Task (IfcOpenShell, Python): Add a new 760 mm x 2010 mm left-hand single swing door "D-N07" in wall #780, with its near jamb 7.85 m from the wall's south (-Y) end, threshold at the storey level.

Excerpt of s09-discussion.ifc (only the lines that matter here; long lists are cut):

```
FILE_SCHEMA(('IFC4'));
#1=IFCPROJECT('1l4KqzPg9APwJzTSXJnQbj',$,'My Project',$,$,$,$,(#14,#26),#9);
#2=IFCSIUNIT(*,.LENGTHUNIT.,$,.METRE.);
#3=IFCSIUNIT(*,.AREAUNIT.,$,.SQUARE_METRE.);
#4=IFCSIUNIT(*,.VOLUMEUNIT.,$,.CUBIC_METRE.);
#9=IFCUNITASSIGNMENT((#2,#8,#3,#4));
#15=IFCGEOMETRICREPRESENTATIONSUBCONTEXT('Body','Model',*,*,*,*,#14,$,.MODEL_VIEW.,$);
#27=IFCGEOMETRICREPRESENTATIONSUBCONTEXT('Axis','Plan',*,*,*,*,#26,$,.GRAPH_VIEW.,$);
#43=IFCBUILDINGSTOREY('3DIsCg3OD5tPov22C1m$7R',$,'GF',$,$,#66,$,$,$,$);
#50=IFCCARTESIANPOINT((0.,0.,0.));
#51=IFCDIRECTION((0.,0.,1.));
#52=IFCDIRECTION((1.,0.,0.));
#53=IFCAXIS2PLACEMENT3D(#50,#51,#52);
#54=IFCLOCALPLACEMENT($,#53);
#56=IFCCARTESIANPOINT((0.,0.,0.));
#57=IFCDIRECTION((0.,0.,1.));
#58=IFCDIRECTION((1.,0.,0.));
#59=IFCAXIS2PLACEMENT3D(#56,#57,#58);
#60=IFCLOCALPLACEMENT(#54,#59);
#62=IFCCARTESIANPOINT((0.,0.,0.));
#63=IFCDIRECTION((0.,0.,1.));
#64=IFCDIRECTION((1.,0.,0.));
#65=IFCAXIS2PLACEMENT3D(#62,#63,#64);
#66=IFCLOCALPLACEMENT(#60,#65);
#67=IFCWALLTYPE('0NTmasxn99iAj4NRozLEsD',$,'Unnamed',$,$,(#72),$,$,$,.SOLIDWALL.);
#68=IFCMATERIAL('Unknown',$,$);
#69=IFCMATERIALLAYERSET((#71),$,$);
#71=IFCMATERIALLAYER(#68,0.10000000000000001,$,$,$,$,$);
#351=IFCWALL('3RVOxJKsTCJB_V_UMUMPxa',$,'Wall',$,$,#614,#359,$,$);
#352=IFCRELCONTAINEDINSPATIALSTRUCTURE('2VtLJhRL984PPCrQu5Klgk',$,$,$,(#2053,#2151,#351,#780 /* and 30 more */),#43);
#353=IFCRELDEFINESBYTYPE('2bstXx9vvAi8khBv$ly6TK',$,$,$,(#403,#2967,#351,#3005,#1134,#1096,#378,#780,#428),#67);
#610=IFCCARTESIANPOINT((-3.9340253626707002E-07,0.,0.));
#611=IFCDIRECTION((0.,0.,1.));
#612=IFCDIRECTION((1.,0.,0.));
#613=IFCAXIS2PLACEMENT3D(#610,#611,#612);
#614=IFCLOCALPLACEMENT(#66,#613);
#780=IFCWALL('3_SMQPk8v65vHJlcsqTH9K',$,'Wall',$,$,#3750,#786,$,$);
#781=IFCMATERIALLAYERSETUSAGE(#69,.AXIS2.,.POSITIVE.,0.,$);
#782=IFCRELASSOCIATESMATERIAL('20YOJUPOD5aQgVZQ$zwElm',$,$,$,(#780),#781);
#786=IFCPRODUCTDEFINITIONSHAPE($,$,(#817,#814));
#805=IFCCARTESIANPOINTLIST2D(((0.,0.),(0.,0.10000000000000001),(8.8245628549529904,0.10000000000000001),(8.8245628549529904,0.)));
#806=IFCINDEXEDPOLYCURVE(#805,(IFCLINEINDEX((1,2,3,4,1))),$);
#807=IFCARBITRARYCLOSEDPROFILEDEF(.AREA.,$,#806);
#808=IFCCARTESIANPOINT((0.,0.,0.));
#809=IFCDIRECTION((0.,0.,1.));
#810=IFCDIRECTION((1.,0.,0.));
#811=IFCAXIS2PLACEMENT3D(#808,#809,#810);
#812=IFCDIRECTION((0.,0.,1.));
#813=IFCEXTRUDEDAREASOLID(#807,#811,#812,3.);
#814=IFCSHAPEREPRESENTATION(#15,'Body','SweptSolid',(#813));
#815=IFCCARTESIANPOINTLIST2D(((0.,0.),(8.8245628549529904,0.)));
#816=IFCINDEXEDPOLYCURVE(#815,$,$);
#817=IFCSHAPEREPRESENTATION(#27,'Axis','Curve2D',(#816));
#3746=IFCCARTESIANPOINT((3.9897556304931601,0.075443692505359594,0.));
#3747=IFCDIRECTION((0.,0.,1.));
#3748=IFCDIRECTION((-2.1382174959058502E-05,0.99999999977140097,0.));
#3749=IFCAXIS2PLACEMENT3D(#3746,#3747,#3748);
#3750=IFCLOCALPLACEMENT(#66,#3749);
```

```python
import numpy as np
import ifcopenshell
import ifcopenshell.api.feature
import ifcopenshell.api.geometry
import ifcopenshell.api.root
import ifcopenshell.api.spatial
import ifcopenshell.geom
import ifcopenshell.util.element
import ifcopenshell.util.placement
import ifcopenshell.util.representation
import ifcopenshell.util.shape
import ifcopenshell.util.unit

model = ifcopenshell.open("s09-discussion.ifc")
unit_scale = ifcopenshell.util.unit.calculate_unit_scale(model)
settings = ifcopenshell.geom.settings()


def volume(element):
    """Net volume in cubic metres, openings subtracted."""
    shape = ifcopenshell.geom.create_shape(settings, element)
    return ifcopenshell.util.shape.get_volume(shape.geometry)


wall = model.by_guid("3_SMQPk8v65vHJlcsqTH9K")
storey = ifcopenshell.util.element.get_container(wall, ifc_class="IfcBuildingStorey")
context = ifcopenshell.util.representation.get_context(model, "Model", "Body", "MODEL_VIEW")
before = volume(wall)

width, height, from_end, sill = 0.76, 2.01, 7.85, 0.0  # metres

# The wall runs along its own X axis, and the end named is its -X end.
wall_shape = ifcopenshell.geom.create_shape(settings, wall)
x, y, z = ifcopenshell.util.shape.get_vertices(wall_shape.geometry).T
start = x.min() + from_end
face, thickness = float(y.min()), float(y.max() - y.min())
wall_matrix = ifcopenshell.util.placement.get_local_placement(wall.ObjectPlacement)
level = ifcopenshell.util.placement.get_local_placement(storey.ObjectPlacement)[2, 3]


def in_wall(x, y):
    """Placement at x, y metres in the wall's axes, at sill height."""
    matrix = wall_matrix.copy()
    matrix[:, 3] = wall_matrix @ np.array([x / unit_scale, y / unit_scale, 0.0, 1.0])
    matrix[2, 3] = level + sill / unit_scale
    return matrix


# Opening: a box that overshoots both wall faces by 50 mm.
opening = ifcopenshell.api.root.create_entity(model, ifc_class="IfcOpeningElement", predefined_type="OPENING")
box = ifcopenshell.api.geometry.add_wall_representation(
    model, context=context, length=width, height=height, thickness=thickness + 0.1
)
ifcopenshell.api.geometry.assign_representation(model, product=opening, representation=box)
ifcopenshell.api.geometry.edit_object_placement(model, product=opening, matrix=in_wall(start, face - 0.05), is_si=False)
ifcopenshell.api.feature.add_feature(model, feature=opening, element=wall)

door = ifcopenshell.api.root.create_entity(model, ifc_class="IfcDoor", name="D-N07", predefined_type="DOOR")
door.OverallWidth, door.OverallHeight = width / unit_scale, height / unit_scale
door.OperationType = "SINGLE_SWING_LEFT"
body = ifcopenshell.api.geometry.add_door_representation(
    model,
    context=context,
    overall_width=door.OverallWidth,
    overall_height=door.OverallHeight,
    operation_type="SINGLE_SWING_LEFT",
    lining_properties={"LiningDepth": thickness / unit_scale, "ThresholdDepth": thickness / unit_scale},
)
ifcopenshell.api.geometry.assign_representation(model, product=door, representation=body)
ifcopenshell.api.spatial.assign_container(model, products=[door], relating_structure=storey)
ifcopenshell.api.feature.add_filling(model, opening=opening, element=door)

# The lining spans the wall, so the door starts at the wall face.
ifcopenshell.api.geometry.edit_object_placement(model, product=door, matrix=in_wall(start, face), is_si=False)

after = volume(wall)

print(f"wall volume {before:.3f} -> {after:.3f} m3")

model.write("s09-discussion_rev.ifc")
```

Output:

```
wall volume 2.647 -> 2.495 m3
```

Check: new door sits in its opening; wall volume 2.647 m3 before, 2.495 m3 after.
